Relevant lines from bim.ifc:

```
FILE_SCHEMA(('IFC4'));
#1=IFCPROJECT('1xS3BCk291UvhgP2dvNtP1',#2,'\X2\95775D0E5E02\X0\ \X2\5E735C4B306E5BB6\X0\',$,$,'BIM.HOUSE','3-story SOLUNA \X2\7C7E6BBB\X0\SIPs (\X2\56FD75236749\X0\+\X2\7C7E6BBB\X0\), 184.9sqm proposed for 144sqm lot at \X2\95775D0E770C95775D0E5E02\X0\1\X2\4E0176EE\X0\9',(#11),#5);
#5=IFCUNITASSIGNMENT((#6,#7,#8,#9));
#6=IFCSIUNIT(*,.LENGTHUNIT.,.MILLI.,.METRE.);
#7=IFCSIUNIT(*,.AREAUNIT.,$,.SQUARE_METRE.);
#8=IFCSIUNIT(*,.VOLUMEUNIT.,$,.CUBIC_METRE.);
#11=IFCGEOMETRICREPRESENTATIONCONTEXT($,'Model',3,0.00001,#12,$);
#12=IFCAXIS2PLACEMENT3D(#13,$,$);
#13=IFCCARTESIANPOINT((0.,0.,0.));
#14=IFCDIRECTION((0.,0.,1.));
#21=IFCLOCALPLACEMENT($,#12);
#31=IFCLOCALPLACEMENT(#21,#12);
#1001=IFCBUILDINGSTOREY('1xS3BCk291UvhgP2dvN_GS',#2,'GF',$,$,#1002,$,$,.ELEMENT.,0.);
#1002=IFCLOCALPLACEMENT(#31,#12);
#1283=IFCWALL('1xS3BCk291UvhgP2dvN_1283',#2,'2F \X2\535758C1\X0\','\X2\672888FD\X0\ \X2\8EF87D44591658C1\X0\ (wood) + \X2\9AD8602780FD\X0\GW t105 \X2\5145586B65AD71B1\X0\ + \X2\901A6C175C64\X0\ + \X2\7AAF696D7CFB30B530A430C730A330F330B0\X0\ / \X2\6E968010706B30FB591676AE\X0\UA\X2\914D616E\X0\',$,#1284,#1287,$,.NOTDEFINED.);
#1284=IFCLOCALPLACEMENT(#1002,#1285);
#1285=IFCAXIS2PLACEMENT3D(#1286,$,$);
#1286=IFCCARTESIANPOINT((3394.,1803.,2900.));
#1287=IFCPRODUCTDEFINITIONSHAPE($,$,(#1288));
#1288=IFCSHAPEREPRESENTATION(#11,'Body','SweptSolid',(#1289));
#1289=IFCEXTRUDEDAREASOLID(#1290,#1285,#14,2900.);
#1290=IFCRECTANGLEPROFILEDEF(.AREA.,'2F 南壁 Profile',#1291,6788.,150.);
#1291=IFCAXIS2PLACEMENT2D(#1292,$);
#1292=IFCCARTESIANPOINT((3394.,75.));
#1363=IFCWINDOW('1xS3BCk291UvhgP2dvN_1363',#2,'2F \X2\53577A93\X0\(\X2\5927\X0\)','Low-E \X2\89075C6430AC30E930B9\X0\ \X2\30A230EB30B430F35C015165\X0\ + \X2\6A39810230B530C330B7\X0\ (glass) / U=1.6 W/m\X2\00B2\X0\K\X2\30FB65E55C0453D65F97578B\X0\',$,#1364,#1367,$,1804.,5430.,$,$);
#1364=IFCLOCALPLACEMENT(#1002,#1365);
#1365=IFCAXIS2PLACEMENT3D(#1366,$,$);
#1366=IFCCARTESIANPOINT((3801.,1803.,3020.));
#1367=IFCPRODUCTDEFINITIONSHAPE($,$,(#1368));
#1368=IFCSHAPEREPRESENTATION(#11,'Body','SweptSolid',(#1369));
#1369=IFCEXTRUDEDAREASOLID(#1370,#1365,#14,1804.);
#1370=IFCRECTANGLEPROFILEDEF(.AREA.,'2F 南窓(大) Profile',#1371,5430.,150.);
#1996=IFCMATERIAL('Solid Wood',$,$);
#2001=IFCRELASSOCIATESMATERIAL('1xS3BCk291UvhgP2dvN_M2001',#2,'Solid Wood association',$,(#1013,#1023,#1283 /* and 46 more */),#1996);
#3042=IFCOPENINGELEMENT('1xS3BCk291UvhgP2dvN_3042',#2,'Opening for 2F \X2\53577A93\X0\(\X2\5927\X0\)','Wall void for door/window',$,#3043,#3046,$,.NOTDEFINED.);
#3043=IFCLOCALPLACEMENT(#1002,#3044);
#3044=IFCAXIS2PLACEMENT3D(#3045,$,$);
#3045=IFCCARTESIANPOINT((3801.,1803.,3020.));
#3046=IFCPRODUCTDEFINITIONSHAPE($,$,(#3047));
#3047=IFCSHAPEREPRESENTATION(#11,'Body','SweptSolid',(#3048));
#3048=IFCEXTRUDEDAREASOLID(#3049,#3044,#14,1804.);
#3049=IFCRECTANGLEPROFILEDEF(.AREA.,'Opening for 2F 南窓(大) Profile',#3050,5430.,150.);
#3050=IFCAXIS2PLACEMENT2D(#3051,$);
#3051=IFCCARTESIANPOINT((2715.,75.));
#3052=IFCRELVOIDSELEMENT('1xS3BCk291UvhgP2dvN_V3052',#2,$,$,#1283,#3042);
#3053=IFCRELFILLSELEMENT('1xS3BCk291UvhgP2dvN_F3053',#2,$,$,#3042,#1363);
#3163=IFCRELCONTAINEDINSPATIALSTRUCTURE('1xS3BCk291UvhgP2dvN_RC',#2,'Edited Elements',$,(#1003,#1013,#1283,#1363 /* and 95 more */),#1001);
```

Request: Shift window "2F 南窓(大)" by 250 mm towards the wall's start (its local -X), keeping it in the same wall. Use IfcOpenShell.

```python
import ifcopenshell
import ifcopenshell.api.geometry
import ifcopenshell.util.placement
import ifcopenshell.util.unit

model = ifcopenshell.open("bim.ifc")
unit_scale = ifcopenshell.util.unit.calculate_unit_scale(model)

window = model.by_id(1363)
opening = window.FillsVoids[0].RelatingOpeningElement
wall = opening.VoidsElements[0].RelatingBuildingElement

wall_matrix = ifcopenshell.util.placement.get_local_placement(wall.ObjectPlacement)
shift = wall_matrix[:3, 0] * -0.25 / unit_scale
before = ifcopenshell.util.placement.get_local_placement(window.ObjectPlacement)[:3, 3].copy()

# The window is not placed relative to its opening, so move both.
for product in (opening, window):
    matrix = ifcopenshell.util.placement.get_local_placement(product.ObjectPlacement)
    matrix[:3, 3] += shift
    ifcopenshell.api.geometry.edit_object_placement(model, product=product, matrix=matrix, is_si=False)

after = ifcopenshell.util.placement.get_local_placement(window.ObjectPlacement)[:3, 3]
print("window moved by", (after - before).round(3) + 0.0)

model.write("bim_rev.ifc")
```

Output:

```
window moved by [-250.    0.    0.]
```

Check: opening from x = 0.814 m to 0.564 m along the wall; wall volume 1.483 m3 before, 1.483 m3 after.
